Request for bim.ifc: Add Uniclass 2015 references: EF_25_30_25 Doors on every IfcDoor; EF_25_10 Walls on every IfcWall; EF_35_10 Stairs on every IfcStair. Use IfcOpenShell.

First a look at what the model holds.

```python
import ifcopenshell

model = ifcopenshell.open("bim.ifc")
print(model.schema)
print("classifications:", [c.Name for c in model.by_type("IfcClassification")])
for ifc_class in ("IfcDoor", "IfcRoof", "IfcStair", "IfcWall", "IfcWindow"):
    print(ifc_class, len(model.by_type(ifc_class)))
```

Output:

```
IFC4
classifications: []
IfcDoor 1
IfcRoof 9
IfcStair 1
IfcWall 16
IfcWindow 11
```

```python
import ifcopenshell
import ifcopenshell.api.classification

model = ifcopenshell.open("bim.ifc")

system = ifcopenshell.api.classification.add_classification(model, classification="Uniclass 2015")

codes = {
    "IfcDoor": ("EF_25_30_25", "Doors"),
    "IfcWall": ("EF_25_10", "Walls"),
    "IfcStair": ("EF_35_10", "Stairs"),
}
for ifc_class, (code, name) in codes.items():
    products = model.by_type(ifc_class)
    ifcopenshell.api.classification.add_reference(
        model, products=products, classification=system, identification=code, name=name
    )
    print(code, len(products))

model.write("bim_rev.ifc")
```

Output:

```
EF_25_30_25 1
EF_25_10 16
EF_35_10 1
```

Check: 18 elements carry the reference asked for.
